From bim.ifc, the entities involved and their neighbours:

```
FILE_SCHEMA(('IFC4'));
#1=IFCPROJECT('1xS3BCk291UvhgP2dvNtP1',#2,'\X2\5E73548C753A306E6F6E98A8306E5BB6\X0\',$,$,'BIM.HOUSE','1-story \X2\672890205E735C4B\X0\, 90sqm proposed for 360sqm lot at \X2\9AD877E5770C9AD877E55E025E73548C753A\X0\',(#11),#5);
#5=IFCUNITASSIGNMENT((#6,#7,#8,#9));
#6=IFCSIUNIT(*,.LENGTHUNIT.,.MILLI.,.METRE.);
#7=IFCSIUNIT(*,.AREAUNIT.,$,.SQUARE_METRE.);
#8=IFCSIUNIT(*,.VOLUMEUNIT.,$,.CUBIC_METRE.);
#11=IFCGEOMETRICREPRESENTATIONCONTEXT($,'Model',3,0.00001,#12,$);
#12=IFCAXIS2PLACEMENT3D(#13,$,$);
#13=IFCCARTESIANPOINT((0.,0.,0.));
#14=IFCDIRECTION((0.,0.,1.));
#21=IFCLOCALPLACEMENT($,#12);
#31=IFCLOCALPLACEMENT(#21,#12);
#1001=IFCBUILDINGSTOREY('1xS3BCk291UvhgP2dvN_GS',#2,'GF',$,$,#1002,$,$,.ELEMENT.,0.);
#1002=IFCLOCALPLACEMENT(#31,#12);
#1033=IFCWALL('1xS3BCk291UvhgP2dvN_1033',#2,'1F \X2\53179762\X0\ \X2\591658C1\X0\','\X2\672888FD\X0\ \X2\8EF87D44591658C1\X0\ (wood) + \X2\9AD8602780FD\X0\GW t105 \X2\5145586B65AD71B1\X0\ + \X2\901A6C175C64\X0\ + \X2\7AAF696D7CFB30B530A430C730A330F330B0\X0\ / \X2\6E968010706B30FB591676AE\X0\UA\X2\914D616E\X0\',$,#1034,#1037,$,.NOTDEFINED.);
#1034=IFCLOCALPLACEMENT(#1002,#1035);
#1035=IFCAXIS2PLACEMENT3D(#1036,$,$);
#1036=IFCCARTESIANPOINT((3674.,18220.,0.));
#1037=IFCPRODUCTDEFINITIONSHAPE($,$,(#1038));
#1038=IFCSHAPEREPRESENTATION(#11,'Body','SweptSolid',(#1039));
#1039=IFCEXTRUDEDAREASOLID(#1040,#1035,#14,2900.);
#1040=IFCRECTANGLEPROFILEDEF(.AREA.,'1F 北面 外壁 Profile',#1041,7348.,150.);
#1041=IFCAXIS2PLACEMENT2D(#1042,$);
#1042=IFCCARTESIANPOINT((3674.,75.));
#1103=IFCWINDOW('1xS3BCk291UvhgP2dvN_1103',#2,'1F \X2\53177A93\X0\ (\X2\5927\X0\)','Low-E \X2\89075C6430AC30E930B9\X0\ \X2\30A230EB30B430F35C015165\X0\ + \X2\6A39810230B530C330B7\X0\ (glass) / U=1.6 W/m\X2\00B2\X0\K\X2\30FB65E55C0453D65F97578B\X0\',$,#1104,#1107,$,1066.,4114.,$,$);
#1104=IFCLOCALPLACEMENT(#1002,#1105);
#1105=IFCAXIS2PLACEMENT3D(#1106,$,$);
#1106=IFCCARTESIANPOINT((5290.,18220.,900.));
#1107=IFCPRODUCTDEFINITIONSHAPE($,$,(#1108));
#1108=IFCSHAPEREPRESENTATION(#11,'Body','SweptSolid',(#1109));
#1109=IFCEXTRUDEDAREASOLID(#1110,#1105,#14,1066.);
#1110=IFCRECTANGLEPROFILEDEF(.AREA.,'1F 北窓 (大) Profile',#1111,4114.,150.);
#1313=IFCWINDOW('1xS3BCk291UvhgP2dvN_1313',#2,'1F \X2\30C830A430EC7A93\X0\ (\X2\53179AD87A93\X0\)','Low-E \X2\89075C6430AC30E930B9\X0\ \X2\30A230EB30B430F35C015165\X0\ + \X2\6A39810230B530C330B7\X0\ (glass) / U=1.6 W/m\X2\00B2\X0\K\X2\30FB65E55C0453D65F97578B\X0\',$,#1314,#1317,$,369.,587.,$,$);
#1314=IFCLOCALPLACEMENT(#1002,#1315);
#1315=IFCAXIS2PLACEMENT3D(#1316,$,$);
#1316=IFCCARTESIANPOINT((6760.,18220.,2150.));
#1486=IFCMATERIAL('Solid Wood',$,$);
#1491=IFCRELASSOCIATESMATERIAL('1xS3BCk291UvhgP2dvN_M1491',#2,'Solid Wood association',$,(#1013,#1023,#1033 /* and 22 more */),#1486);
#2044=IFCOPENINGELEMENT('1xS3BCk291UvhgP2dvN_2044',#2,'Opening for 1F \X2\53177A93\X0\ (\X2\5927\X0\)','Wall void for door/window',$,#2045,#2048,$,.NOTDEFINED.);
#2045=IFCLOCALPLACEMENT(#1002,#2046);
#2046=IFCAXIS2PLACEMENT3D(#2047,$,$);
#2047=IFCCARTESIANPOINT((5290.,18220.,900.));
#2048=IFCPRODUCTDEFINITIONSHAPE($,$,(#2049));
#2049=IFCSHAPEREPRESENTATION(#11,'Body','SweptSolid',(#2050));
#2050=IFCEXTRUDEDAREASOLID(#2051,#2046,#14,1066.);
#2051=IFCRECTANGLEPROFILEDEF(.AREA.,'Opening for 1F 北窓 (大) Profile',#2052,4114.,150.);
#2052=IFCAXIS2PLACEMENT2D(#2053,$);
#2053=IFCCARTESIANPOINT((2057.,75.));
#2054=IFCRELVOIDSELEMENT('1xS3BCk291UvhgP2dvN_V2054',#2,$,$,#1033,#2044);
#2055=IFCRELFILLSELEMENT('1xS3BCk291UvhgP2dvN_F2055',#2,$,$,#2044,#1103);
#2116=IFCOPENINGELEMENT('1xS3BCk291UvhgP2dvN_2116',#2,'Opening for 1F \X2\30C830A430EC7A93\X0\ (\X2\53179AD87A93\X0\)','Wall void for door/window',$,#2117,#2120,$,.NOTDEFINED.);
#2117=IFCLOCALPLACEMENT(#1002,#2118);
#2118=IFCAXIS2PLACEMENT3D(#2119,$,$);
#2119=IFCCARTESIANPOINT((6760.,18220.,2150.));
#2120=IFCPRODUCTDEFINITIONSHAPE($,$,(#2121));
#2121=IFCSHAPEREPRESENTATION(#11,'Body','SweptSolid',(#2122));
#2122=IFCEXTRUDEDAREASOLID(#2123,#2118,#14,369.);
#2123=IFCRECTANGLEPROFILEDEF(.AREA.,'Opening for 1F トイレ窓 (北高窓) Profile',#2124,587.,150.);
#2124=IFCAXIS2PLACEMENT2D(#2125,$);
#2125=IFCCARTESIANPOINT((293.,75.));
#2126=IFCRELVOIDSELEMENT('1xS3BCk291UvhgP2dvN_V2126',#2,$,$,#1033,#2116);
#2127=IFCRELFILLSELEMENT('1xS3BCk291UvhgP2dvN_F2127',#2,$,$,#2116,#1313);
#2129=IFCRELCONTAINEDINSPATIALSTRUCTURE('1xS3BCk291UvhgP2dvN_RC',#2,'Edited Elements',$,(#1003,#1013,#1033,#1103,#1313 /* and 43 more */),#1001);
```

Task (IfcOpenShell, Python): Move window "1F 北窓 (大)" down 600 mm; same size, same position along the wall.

```python
import numpy as np
import ifcopenshell
import ifcopenshell.api.geometry
import ifcopenshell.util.placement
import ifcopenshell.util.unit

model = ifcopenshell.open("bim.ifc")
unit_scale = ifcopenshell.util.unit.calculate_unit_scale(model)

window = model.by_guid("1xS3BCk291UvhgP2dvN_1103")
opening = window.FillsVoids[0].RelatingOpeningElement
dz = -600.0

shift = np.array([0.0, 0.0, dz])
# The window is not placed relative to its opening, so move both.
for product in (opening, window):
    matrix = ifcopenshell.util.placement.get_local_placement(product.ObjectPlacement)
    matrix[:3, 3] += shift
    ifcopenshell.api.geometry.edit_object_placement(model, product=product, matrix=matrix, is_si=False)

print(f"moved by {dz * unit_scale:+.3f} m")

model.write("bim_updated.ifc")
```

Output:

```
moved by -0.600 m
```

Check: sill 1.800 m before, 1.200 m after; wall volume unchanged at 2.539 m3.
